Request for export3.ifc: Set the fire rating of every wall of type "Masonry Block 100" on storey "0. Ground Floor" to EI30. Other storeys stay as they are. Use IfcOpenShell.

First a look at what the model holds.

```python
import ifcopenshell
import ifcopenshell.util.element

model = ifcopenshell.open("export3.ifc")
print(model.schema)
storey = next(s for s in model.by_type("IfcBuildingStorey") if s.Name == "0. Ground Floor")
walls = [e for e in ifcopenshell.util.element.get_decomposition(storey) if e.is_a("IfcWall")]
seen = {}
for e in walls:
    element_type = ifcopenshell.util.element.get_type(e)
    key = (element_type.Name if element_type != e and element_type else None, ifcopenshell.util.element.get_pset(e, "Pset_WallCommon", "FireRating"))
    seen[key] = seen.get(key, 0) + 1
for (name, value), count in sorted(seen.items(), key=str):
    print(count, "x", name, "|", value)
```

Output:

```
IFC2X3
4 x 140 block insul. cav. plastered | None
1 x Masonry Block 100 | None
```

```python
import ifcopenshell
import ifcopenshell.api.pset
import ifcopenshell.util.element

model = ifcopenshell.open("export3.ifc")

storey = next(s for s in model.by_type("IfcBuildingStorey") if s.Name == "0. Ground Floor")
walls = [e for e in ifcopenshell.util.element.get_decomposition(storey) if e.is_a("IfcWall")]

count = 0
for e in walls:
    element_type = ifcopenshell.util.element.get_type(e)
    if element_type in (None, e) or element_type.Name != "Masonry Block 100":
        continue
    # add_pset returns the element's existing set when there is one.
    pset = ifcopenshell.api.pset.add_pset(model, product=e, name="Pset_WallCommon")
    ifcopenshell.api.pset.edit_pset(model, pset=pset, properties={"FireRating": "EI30"})
    count += 1

print(count, "walls updated")

model.write("export3_rev.ifc")
```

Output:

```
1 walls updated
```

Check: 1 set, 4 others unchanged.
